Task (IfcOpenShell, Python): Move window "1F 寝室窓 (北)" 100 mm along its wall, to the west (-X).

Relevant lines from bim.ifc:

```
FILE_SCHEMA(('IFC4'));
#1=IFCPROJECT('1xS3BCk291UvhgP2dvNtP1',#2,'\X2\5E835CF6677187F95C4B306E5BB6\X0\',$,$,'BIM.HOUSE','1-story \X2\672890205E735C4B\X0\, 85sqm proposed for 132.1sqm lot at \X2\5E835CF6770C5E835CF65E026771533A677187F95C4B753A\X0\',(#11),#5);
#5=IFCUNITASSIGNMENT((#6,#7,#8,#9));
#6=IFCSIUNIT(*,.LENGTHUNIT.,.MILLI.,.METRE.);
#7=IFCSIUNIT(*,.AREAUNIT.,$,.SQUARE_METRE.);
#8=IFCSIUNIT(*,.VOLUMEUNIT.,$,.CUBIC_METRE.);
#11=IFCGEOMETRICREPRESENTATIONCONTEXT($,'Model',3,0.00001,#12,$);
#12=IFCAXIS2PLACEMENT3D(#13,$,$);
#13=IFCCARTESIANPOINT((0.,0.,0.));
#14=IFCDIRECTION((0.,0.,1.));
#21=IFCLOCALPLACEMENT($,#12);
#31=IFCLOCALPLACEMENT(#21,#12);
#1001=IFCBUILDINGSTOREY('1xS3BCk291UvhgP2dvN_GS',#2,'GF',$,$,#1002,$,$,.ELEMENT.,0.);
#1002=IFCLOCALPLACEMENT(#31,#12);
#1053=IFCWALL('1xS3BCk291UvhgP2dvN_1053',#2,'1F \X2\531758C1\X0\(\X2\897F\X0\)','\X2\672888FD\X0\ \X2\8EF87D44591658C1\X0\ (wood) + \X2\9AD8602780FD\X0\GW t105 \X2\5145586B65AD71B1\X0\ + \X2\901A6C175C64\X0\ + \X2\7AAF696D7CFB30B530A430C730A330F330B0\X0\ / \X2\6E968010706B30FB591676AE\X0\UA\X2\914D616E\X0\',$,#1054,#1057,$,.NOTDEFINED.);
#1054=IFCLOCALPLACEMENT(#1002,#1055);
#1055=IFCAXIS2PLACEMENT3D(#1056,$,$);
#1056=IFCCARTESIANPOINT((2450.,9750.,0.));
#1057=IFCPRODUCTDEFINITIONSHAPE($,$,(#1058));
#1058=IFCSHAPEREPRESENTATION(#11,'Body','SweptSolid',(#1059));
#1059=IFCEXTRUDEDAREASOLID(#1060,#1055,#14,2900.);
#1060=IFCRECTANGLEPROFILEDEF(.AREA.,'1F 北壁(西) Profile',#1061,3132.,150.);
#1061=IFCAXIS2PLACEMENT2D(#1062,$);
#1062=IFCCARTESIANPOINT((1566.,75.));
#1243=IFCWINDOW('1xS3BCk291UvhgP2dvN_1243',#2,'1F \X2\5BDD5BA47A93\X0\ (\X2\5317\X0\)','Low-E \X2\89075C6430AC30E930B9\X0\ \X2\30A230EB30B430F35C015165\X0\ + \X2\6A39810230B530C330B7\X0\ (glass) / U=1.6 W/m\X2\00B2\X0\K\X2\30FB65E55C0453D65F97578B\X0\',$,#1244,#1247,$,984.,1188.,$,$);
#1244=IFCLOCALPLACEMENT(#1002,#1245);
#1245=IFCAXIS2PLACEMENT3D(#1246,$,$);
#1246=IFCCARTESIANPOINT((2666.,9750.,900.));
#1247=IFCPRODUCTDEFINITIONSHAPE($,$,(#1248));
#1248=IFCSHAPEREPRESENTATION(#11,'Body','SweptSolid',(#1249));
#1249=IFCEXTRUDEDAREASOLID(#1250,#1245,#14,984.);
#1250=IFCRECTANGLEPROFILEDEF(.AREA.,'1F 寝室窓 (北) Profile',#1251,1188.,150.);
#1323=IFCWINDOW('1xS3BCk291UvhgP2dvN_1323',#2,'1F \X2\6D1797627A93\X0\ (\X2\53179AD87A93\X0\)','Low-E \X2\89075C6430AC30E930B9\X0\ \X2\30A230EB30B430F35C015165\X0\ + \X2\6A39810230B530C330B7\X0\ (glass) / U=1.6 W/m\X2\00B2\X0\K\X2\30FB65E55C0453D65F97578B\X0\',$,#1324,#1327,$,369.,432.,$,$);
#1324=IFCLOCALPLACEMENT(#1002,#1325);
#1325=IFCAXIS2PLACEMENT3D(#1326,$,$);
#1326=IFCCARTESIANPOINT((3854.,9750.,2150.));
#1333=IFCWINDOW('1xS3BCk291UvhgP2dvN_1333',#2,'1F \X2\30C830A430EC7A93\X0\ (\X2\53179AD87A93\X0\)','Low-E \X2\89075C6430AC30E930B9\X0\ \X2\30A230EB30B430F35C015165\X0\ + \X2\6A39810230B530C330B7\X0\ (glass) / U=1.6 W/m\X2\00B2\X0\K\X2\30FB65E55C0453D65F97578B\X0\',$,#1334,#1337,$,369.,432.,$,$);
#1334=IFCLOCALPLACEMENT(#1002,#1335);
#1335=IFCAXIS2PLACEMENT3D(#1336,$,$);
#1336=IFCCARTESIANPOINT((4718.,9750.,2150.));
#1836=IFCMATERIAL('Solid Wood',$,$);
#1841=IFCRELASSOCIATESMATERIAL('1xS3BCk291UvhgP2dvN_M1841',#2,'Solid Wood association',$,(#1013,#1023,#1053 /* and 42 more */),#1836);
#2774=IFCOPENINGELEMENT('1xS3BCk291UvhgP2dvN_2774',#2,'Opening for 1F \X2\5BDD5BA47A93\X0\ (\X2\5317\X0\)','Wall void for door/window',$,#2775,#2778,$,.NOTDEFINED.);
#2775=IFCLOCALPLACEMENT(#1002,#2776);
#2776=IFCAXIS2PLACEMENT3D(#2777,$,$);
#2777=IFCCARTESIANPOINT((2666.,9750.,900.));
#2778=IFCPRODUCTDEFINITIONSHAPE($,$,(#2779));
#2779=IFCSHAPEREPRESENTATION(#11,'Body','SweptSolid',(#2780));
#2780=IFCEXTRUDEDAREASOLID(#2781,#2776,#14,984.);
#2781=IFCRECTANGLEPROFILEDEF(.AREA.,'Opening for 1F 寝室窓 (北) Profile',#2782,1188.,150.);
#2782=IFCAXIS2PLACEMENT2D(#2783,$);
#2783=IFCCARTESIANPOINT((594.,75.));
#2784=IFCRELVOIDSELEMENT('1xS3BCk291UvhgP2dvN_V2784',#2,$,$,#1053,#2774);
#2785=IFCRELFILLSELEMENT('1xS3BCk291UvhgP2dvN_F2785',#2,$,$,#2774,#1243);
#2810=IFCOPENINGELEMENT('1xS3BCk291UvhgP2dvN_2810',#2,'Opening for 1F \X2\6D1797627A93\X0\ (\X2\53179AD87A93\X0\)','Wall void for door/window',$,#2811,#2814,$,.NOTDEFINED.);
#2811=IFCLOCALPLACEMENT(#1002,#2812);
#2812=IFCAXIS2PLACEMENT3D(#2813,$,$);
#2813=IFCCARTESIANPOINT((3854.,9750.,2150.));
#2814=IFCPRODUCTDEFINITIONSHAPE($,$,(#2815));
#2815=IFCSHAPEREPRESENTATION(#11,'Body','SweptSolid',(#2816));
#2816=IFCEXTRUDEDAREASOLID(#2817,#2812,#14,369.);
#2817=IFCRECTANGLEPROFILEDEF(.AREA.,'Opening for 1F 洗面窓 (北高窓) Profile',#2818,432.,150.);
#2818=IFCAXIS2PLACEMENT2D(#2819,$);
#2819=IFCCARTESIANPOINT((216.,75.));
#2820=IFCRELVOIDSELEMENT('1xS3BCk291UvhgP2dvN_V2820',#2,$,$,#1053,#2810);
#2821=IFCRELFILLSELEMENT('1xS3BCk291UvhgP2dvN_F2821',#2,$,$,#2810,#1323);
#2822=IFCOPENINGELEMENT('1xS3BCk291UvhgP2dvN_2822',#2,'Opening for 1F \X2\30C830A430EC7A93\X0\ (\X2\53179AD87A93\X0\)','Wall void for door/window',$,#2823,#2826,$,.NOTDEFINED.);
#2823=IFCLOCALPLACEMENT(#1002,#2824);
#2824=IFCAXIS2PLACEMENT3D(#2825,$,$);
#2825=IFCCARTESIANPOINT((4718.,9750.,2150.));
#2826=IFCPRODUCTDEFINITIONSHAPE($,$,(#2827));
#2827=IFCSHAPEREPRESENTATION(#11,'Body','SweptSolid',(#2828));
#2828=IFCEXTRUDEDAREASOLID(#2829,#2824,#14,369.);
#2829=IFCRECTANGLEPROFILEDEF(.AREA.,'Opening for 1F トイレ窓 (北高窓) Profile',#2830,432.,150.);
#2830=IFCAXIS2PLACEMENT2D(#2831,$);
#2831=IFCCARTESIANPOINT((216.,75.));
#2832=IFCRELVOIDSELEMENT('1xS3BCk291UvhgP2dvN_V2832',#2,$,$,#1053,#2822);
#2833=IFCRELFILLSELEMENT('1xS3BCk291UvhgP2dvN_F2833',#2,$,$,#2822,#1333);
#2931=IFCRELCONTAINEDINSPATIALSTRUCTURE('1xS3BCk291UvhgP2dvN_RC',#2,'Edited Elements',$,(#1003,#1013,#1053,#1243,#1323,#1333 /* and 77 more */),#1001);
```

```python
import ifcopenshell
import ifcopenshell.api.geometry
import ifcopenshell.util.placement
import ifcopenshell.util.unit

model = ifcopenshell.open("bim.ifc")
unit_scale = ifcopenshell.util.unit.calculate_unit_scale(model)

window = model.by_guid("1xS3BCk291UvhgP2dvN_1243")
opening = window.FillsVoids[0].RelatingOpeningElement
wall = opening.VoidsElements[0].RelatingBuildingElement

wall_matrix = ifcopenshell.util.placement.get_local_placement(wall.ObjectPlacement)
shift = wall_matrix[:3, 0] * -0.1 / unit_scale
before = ifcopenshell.util.placement.get_local_placement(window.ObjectPlacement)[:3, 3].copy()

# The window is not placed relative to its opening, so move both.
for product in (opening, window):
    matrix = ifcopenshell.util.placement.get_local_placement(product.ObjectPlacement)
    matrix[:3, 3] += shift
    ifcopenshell.api.geometry.edit_object_placement(model, product=product, matrix=matrix, is_si=False)

after = ifcopenshell.util.placement.get_local_placement(window.ObjectPlacement)[:3, 3]
print("window moved by", (after - before).round(3) + 0.0)

model.write("bim_updated.ifc")
```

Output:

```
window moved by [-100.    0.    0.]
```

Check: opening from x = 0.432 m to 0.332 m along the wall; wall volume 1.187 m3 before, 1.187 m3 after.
